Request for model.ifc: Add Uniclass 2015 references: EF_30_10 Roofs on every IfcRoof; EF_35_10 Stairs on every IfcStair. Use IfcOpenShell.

First a look at what the model holds.

```python
import ifcopenshell

model = ifcopenshell.open("model.ifc")
print(model.schema)
print("classifications:", [c.Name for c in model.by_type("IfcClassification")])
for ifc_class in ("IfcDoor", "IfcRoof", "IfcStair", "IfcWall", "IfcWindow"):
    print(ifc_class, len(model.by_type(ifc_class)))
```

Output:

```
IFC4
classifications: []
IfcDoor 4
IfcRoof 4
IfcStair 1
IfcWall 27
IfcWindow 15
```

```python
import ifcopenshell
import ifcopenshell.api.classification

model = ifcopenshell.open("model.ifc")

system = ifcopenshell.api.classification.add_classification(model, classification="Uniclass 2015")

codes = {
    "IfcRoof": ("EF_30_10", "Roofs"),
    "IfcStair": ("EF_35_10", "Stairs"),
}
for ifc_class, (code, name) in codes.items():
    products = model.by_type(ifc_class)
    ifcopenshell.api.classification.add_reference(
        model, products=products, classification=system, identification=code, name=name
    )
    print(code, len(products))

model.write("model_updated.ifc")
```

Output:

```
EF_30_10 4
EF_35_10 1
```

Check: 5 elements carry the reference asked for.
